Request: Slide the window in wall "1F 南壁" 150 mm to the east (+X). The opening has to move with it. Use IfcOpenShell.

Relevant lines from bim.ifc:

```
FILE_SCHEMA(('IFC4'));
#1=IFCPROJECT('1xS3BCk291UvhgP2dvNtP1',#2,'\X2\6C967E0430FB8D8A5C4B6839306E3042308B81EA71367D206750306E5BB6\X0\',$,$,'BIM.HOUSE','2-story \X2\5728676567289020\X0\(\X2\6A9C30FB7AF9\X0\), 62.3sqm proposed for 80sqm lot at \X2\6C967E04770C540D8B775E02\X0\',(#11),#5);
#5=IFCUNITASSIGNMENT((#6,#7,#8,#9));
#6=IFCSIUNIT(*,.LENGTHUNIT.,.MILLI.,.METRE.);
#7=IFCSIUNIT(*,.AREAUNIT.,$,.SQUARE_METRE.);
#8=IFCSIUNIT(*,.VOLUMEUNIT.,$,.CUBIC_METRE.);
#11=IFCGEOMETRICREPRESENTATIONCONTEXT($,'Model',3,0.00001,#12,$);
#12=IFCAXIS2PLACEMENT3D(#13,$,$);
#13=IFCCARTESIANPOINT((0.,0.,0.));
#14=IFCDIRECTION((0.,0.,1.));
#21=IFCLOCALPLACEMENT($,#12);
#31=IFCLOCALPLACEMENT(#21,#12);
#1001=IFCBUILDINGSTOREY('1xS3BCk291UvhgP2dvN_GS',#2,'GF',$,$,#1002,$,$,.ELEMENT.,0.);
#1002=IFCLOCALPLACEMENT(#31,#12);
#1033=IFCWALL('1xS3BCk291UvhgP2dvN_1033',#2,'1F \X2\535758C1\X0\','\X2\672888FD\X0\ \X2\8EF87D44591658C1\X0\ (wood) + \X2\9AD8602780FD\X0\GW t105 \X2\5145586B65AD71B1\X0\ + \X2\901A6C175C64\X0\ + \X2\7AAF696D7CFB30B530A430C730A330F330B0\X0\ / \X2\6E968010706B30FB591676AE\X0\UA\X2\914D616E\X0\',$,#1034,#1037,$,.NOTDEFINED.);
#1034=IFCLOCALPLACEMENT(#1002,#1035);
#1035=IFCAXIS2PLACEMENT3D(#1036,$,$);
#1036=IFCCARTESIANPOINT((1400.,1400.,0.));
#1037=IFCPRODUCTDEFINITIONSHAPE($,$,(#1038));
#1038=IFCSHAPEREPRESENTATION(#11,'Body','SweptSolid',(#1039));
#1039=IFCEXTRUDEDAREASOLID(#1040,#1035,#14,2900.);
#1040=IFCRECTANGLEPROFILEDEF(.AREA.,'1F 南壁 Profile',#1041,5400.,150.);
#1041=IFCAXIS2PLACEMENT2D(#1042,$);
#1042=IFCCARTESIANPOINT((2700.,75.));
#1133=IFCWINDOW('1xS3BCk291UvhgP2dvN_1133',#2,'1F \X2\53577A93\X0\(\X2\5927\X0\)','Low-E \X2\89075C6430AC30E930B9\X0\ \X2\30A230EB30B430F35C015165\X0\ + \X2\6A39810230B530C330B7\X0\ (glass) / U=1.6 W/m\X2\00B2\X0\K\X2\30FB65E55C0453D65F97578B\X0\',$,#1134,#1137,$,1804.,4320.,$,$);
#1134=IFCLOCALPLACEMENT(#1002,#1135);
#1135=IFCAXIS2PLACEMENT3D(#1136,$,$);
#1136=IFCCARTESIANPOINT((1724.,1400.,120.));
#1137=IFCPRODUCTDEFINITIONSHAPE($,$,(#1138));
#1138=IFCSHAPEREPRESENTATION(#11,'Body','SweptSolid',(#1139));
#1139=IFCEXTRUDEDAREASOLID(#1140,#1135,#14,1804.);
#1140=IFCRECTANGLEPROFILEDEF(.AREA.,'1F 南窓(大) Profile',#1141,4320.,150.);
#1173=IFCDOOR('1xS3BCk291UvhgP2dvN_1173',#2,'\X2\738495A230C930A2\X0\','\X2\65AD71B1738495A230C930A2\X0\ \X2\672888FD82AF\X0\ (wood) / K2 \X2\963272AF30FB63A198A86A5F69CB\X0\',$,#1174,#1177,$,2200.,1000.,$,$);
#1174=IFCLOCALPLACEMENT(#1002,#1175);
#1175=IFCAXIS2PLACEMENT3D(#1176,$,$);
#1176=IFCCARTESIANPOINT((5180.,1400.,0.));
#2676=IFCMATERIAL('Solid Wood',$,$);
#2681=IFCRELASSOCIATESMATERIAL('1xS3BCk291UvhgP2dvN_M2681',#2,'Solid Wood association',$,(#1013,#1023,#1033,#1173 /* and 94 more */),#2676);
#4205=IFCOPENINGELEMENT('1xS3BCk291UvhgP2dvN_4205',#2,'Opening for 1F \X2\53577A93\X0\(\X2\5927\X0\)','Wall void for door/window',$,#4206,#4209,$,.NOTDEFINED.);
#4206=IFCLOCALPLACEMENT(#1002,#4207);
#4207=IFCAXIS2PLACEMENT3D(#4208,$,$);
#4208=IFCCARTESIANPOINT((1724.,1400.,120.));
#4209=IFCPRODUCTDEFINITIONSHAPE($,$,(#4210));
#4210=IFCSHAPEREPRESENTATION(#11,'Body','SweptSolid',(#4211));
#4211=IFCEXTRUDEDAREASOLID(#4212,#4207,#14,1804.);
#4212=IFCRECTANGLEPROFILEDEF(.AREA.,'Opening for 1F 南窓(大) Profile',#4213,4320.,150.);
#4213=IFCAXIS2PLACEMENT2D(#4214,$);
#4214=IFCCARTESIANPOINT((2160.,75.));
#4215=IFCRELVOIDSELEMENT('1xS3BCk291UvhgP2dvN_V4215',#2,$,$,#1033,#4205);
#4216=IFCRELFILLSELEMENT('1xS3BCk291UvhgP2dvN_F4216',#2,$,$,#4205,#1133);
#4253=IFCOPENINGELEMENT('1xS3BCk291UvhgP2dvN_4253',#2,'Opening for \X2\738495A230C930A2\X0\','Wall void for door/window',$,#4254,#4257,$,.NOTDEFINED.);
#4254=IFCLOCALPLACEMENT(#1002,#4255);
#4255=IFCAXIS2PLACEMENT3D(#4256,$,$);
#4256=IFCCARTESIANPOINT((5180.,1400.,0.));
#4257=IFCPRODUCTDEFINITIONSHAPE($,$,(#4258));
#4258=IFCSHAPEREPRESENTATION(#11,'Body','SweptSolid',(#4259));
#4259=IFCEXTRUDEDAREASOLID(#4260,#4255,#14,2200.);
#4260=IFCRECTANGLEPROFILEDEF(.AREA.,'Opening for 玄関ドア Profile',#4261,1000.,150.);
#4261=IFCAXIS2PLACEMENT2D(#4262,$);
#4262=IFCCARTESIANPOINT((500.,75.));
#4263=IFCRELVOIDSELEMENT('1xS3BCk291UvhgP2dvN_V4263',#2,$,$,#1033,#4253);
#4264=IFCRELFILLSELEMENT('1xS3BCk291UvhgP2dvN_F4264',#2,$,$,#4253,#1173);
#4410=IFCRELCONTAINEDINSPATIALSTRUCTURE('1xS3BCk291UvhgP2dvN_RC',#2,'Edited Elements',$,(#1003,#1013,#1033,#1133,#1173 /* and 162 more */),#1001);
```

```python
import ifcopenshell
import ifcopenshell.api.geometry
import ifcopenshell.util.placement
import ifcopenshell.util.unit

model = ifcopenshell.open("bim.ifc")
unit_scale = ifcopenshell.util.unit.calculate_unit_scale(model)

window = model.by_guid("1xS3BCk291UvhgP2dvN_1133")
opening = window.FillsVoids[0].RelatingOpeningElement
wall = opening.VoidsElements[0].RelatingBuildingElement

wall_matrix = ifcopenshell.util.placement.get_local_placement(wall.ObjectPlacement)
shift = wall_matrix[:3, 0] * 0.15 / unit_scale
before = ifcopenshell.util.placement.get_local_placement(window.ObjectPlacement)[:3, 3].copy()

# The window is not placed relative to its opening, so move both.
for product in (opening, window):
    matrix = ifcopenshell.util.placement.get_local_placement(product.ObjectPlacement)
    matrix[:3, 3] += shift
    ifcopenshell.api.geometry.edit_object_placement(model, product=product, matrix=matrix, is_si=False)

after = ifcopenshell.util.placement.get_local_placement(window.ObjectPlacement)[:3, 3]
print("window moved by", (after - before).round(3) + 0.0)

model.write("bim_rev.ifc")
```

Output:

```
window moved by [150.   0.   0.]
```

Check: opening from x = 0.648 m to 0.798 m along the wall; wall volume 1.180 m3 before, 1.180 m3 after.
